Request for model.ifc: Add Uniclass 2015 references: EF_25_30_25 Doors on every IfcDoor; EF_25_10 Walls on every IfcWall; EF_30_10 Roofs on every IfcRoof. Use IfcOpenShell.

First a look at what the model holds.

```python
import ifcopenshell

model = ifcopenshell.open("model.ifc")
print(model.schema)
print("classifications:", [c.Name for c in model.by_type("IfcClassification")])
for ifc_class in ("IfcDoor", "IfcRoof", "IfcStair", "IfcWall", "IfcWindow"):
    print(ifc_class, len(model.by_type(ifc_class)))
```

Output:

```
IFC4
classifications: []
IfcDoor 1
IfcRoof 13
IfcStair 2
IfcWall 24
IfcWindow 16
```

```python
import ifcopenshell
import ifcopenshell.api.classification

model = ifcopenshell.open("model.ifc")

system = ifcopenshell.api.classification.add_classification(model, classification="Uniclass 2015")

codes = {
    "IfcDoor": ("EF_25_30_25", "Doors"),
    "IfcWall": ("EF_25_10", "Walls"),
    "IfcRoof": ("EF_30_10", "Roofs"),
}
for ifc_class, (code, name) in codes.items():
    products = model.by_type(ifc_class)
    ifcopenshell.api.classification.add_reference(
        model, products=products, classification=system, identification=code, name=name
    )
    print(code, len(products))

model.write("model-out.ifc")
```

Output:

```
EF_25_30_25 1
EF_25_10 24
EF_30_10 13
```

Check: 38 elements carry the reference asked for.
